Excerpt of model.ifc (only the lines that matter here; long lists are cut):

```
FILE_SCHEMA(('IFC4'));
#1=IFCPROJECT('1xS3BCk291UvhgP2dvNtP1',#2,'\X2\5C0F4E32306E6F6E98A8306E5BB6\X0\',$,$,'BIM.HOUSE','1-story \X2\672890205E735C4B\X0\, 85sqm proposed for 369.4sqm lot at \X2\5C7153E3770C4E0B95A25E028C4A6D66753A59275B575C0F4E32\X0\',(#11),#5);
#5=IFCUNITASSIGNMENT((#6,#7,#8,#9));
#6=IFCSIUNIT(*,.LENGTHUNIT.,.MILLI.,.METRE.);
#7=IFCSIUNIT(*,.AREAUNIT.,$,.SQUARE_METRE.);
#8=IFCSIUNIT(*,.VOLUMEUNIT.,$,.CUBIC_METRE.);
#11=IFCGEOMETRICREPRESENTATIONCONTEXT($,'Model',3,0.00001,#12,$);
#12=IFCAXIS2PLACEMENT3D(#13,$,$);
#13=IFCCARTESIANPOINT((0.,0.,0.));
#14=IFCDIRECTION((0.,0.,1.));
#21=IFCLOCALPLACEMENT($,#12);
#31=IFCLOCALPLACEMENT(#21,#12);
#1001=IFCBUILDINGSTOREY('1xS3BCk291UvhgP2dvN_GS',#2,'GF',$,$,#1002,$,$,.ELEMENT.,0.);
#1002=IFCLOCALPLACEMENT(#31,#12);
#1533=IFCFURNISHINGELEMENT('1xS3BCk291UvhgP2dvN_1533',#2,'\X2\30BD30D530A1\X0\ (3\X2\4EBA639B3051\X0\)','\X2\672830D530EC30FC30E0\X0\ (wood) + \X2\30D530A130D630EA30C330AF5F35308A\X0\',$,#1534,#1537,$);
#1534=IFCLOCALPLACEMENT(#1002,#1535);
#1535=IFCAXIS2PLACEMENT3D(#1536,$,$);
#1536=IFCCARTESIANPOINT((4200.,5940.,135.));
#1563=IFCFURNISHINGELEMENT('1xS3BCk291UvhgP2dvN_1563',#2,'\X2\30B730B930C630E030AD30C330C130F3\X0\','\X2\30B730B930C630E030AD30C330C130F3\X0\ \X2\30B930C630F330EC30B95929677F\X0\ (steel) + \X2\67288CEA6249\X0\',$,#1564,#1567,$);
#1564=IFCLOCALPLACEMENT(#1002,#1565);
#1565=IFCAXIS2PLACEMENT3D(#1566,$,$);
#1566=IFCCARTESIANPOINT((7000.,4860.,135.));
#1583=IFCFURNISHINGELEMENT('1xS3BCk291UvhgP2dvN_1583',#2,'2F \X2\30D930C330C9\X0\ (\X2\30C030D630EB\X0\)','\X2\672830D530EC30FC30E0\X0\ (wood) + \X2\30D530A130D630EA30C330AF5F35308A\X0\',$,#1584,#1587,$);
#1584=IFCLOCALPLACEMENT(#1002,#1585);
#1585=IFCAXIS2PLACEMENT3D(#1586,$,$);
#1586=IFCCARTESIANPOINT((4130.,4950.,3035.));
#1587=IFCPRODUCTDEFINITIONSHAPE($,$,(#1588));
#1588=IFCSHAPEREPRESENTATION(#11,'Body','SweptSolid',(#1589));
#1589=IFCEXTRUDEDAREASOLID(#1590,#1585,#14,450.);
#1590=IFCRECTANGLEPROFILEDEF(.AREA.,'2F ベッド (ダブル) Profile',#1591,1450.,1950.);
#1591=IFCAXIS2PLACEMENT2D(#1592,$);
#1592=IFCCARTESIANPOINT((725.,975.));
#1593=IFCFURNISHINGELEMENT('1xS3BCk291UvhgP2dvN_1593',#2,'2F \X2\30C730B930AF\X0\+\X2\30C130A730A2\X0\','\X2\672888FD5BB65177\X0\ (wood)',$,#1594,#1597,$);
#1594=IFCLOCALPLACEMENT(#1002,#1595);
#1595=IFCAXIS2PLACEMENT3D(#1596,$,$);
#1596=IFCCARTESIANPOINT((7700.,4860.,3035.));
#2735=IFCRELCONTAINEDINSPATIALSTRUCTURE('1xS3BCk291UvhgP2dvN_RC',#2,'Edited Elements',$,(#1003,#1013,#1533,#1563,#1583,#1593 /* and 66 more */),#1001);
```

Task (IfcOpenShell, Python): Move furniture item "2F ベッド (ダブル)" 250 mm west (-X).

```python
import ifcopenshell
import ifcopenshell.api.geometry
import ifcopenshell.util.placement
import ifcopenshell.util.unit

model = ifcopenshell.open("model.ifc")
unit_scale = ifcopenshell.util.unit.calculate_unit_scale(model)

item = model.by_id(1583)
matrix = ifcopenshell.util.placement.get_local_placement(item.ObjectPlacement)
matrix[0, 3] -= 0.25 / unit_scale
ifcopenshell.api.geometry.edit_object_placement(model, product=item, matrix=matrix, is_si=False)

print(ifcopenshell.util.placement.get_local_placement(item.ObjectPlacement).round(3) + 0.0)

model.write("model_v2.ifc")
```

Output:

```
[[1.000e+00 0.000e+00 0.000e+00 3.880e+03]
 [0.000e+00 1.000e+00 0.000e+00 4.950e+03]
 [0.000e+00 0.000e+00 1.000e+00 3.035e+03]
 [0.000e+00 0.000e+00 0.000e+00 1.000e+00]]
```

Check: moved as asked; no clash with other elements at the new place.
